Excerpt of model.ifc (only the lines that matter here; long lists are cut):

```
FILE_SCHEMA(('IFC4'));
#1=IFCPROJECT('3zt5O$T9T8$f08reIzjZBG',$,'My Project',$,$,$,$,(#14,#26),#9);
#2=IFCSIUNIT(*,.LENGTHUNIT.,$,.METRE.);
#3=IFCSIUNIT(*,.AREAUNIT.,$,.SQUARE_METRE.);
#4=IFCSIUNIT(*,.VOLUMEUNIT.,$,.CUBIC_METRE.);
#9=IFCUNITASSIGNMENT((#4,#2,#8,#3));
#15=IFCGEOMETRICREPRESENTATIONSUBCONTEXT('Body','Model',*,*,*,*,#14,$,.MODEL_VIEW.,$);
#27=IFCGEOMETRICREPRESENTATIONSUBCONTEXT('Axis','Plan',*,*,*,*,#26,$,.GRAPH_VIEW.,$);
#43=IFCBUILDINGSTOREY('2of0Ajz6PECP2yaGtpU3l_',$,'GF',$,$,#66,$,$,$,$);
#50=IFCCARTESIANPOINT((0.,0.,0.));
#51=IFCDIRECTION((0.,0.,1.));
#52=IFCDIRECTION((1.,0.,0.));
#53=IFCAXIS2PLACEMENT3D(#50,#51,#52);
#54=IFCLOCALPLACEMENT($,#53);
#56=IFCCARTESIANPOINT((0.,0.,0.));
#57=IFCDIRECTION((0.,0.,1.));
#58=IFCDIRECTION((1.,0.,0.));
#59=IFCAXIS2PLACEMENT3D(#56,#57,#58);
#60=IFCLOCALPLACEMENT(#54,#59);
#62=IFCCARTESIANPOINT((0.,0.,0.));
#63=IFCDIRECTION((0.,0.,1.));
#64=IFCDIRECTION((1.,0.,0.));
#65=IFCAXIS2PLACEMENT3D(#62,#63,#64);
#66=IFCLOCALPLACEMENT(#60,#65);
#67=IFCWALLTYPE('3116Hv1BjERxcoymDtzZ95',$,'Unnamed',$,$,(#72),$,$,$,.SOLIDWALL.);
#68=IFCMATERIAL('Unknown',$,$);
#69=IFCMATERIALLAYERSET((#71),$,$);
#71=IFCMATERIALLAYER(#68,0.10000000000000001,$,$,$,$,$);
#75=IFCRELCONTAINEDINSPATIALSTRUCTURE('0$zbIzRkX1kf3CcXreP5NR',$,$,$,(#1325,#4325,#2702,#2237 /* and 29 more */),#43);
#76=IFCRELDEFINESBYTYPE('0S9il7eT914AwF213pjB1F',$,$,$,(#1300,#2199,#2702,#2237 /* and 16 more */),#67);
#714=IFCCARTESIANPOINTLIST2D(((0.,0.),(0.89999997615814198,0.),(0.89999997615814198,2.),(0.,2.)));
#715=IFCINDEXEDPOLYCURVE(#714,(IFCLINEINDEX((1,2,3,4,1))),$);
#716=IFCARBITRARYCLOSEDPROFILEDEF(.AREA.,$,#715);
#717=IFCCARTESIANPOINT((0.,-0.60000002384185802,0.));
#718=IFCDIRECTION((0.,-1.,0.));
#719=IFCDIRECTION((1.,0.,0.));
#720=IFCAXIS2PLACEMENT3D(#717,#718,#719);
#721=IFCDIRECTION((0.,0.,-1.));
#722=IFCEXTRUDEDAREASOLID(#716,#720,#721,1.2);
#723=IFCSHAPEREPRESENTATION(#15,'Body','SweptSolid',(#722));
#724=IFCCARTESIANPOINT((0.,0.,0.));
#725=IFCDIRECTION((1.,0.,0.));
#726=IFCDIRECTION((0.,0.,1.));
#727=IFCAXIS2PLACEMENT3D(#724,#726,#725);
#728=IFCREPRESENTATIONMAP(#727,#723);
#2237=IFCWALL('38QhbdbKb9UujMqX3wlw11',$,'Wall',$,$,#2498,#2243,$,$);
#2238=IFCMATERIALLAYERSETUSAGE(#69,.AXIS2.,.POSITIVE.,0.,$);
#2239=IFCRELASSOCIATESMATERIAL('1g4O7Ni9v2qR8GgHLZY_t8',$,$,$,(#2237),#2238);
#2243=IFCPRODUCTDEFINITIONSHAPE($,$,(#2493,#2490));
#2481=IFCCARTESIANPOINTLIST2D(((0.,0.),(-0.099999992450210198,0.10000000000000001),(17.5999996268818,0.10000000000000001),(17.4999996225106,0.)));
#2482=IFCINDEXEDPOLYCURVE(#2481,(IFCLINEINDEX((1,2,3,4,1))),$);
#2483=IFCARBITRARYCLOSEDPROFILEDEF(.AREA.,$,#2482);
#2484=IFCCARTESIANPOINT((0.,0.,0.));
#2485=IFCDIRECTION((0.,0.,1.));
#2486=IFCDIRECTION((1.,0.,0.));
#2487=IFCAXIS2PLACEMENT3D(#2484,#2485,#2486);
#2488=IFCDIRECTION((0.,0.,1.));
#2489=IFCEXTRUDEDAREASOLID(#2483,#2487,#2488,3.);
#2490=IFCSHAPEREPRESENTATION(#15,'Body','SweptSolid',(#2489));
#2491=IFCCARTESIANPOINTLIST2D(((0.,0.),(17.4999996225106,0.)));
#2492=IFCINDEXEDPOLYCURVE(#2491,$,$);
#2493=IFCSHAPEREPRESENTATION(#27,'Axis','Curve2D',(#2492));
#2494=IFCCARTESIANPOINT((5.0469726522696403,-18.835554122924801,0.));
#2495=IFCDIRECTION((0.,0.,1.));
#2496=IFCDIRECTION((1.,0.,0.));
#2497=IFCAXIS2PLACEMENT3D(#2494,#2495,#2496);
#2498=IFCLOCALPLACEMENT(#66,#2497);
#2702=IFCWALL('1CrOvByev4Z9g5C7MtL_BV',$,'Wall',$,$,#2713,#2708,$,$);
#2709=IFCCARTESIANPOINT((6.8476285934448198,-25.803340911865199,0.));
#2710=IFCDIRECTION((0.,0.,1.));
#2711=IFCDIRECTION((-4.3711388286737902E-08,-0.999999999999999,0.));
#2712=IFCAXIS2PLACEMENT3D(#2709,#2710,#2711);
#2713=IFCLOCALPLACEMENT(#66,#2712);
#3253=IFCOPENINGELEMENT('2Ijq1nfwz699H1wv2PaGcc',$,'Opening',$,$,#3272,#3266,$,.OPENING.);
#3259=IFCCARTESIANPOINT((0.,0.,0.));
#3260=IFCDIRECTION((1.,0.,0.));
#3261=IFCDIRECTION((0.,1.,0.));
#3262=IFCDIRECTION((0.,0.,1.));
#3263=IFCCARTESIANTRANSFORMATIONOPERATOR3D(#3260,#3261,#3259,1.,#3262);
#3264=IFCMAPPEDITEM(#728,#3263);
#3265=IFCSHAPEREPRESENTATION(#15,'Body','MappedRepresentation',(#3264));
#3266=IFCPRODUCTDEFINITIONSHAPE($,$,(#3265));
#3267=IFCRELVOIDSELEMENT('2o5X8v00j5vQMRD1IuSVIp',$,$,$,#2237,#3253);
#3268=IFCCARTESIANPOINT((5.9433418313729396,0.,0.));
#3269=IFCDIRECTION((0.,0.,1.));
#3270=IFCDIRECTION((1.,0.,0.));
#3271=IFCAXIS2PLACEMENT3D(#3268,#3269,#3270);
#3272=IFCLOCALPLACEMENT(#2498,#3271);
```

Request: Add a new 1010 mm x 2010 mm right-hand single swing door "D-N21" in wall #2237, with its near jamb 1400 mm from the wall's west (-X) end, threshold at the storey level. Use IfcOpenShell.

```python
import numpy as np
import ifcopenshell
import ifcopenshell.api.feature
import ifcopenshell.api.geometry
import ifcopenshell.api.root
import ifcopenshell.api.spatial
import ifcopenshell.geom
import ifcopenshell.util.element
import ifcopenshell.util.placement
import ifcopenshell.util.representation
import ifcopenshell.util.shape
import ifcopenshell.util.unit

model = ifcopenshell.open("model.ifc")
unit_scale = ifcopenshell.util.unit.calculate_unit_scale(model)
settings = ifcopenshell.geom.settings()


def volume(element):
    """Net volume in cubic metres, openings subtracted."""
    shape = ifcopenshell.geom.create_shape(settings, element)
    return ifcopenshell.util.shape.get_volume(shape.geometry)


wall = model.by_id(2237)
storey = ifcopenshell.util.element.get_container(wall, ifc_class="IfcBuildingStorey")
context = ifcopenshell.util.representation.get_context(model, "Model", "Body", "MODEL_VIEW")
before = volume(wall)

width, height, from_end, sill = 1.01, 2.01, 1.4, 0.0  # metres

# The wall runs along its own X axis, and the end named is its -X end.
wall_shape = ifcopenshell.geom.create_shape(settings, wall)
x, y, z = ifcopenshell.util.shape.get_vertices(wall_shape.geometry).T
start = x.min() + from_end
face, thickness = float(y.min()), float(y.max() - y.min())
wall_matrix = ifcopenshell.util.placement.get_local_placement(wall.ObjectPlacement)
level = ifcopenshell.util.placement.get_local_placement(storey.ObjectPlacement)[2, 3]


def in_wall(x, y):
    """Placement at x, y metres in the wall's axes, at sill height."""
    matrix = wall_matrix.copy()
    matrix[:, 3] = wall_matrix @ np.array([x / unit_scale, y / unit_scale, 0.0, 1.0])
    matrix[2, 3] = level + sill / unit_scale
    return matrix


# Opening: a box that overshoots both wall faces by 50 mm.
opening = ifcopenshell.api.root.create_entity(model, ifc_class="IfcOpeningElement", predefined_type="OPENING")
box = ifcopenshell.api.geometry.add_wall_representation(
    model, context=context, length=width, height=height, thickness=thickness + 0.1
)
ifcopenshell.api.geometry.assign_representation(model, product=opening, representation=box)
ifcopenshell.api.geometry.edit_object_placement(model, product=opening, matrix=in_wall(start, face - 0.05), is_si=False)
ifcopenshell.api.feature.add_feature(model, feature=opening, element=wall)

door = ifcopenshell.api.root.create_entity(model, ifc_class="IfcDoor", name="D-N21", predefined_type="DOOR")
door.OverallWidth, door.OverallHeight = width / unit_scale, height / unit_scale
door.OperationType = "SINGLE_SWING_RIGHT"
body = ifcopenshell.api.geometry.add_door_representation(
    model,
    context=context,
    overall_width=door.OverallWidth,
    overall_height=door.OverallHeight,
    operation_type="SINGLE_SWING_RIGHT",
    lining_properties={"LiningDepth": thickness / unit_scale, "ThresholdDepth": thickness / unit_scale},
)
ifcopenshell.api.geometry.assign_representation(model, product=door, representation=body)
ifcopenshell.api.spatial.assign_container(model, products=[door], relating_structure=storey)
ifcopenshell.api.feature.add_filling(model, opening=opening, element=door)

# The lining spans the wall, so the door starts at the wall face.
ifcopenshell.api.geometry.edit_object_placement(model, product=door, matrix=in_wall(start, face), is_si=False)

after = volume(wall)

print(f"wall volume {before:.3f} -> {after:.3f} m3")

model.write("model-out.ifc")
```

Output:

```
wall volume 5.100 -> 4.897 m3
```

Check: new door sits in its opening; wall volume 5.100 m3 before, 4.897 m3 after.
